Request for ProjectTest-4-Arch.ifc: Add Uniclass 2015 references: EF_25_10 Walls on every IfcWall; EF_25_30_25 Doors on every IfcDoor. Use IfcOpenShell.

First a look at what the model holds.

```python
import ifcopenshell

model = ifcopenshell.open("ProjectTest-4-Arch.ifc")
print(model.schema)
print("classifications:", [c.Name for c in model.by_type("IfcClassification")])
for ifc_class in ("IfcDoor", "IfcRoof", "IfcStair", "IfcWall", "IfcWindow"):
    print(ifc_class, len(model.by_type(ifc_class)))
```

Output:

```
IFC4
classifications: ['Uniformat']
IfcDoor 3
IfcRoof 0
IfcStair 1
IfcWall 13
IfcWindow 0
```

```python
import ifcopenshell
import ifcopenshell.api.classification

model = ifcopenshell.open("ProjectTest-4-Arch.ifc")

system = ifcopenshell.api.classification.add_classification(model, classification="Uniclass 2015")

codes = {
    "IfcWall": ("EF_25_10", "Walls"),
    "IfcDoor": ("EF_25_30_25", "Doors"),
}
for ifc_class, (code, name) in codes.items():
    products = model.by_type(ifc_class)
    ifcopenshell.api.classification.add_reference(
        model, products=products, classification=system, identification=code, name=name
    )
    print(code, len(products))

model.write("ProjectTest-4-Arch_rev.ifc")
```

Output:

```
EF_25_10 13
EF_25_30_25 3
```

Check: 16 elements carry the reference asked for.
